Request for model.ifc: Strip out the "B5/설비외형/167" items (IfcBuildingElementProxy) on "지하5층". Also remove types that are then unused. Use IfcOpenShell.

First a look at what the model holds.

```python
import ifcopenshell
import ifcopenshell.util.element

model = ifcopenshell.open("model.ifc")
print(model.schema)
storey = next(s for s in model.by_type("IfcBuildingStorey") if s.Name == "지하5층")
proxies = [e for e in ifcopenshell.util.element.get_decomposition(storey) if e.is_a("IfcBuildingElementProxy")]
seen = {}
for e in proxies:
    element_type = ifcopenshell.util.element.get_type(e)
    name = element_type.Name if element_type not in (None, e) else None
    seen[name] = seen.get(name, 0) + 1
for name, count in sorted(seen.items(), key=str):
    print(count, "x", name)
```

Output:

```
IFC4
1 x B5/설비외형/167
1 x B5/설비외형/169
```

```python
import ifcopenshell
import ifcopenshell.api.root
import ifcopenshell.util.element

model = ifcopenshell.open("model.ifc")

storey = next(s for s in model.by_type("IfcBuildingStorey") if s.Name == "지하5층")
proxies = [e for e in ifcopenshell.util.element.get_decomposition(storey) if e.is_a("IfcBuildingElementProxy")]
targets = [e for e in proxies if (t := ifcopenshell.util.element.get_type(e)) not in (None, e) and t.Name == "B5/설비외형/167"]
types = {ifcopenshell.util.element.get_type(e) for e in targets} - {None, *targets}

for e in targets:
    ifcopenshell.api.root.remove_product(model, product=e)
print(len(targets), "removed")

unused = [t for t in types if not ifcopenshell.util.element.get_types(t)]
for t in unused:
    ifcopenshell.api.root.remove_product(model, product=t)
print(len(unused), "unused types removed")

model.write("model_edited.ifc")
```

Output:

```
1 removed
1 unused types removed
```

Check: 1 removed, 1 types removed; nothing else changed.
